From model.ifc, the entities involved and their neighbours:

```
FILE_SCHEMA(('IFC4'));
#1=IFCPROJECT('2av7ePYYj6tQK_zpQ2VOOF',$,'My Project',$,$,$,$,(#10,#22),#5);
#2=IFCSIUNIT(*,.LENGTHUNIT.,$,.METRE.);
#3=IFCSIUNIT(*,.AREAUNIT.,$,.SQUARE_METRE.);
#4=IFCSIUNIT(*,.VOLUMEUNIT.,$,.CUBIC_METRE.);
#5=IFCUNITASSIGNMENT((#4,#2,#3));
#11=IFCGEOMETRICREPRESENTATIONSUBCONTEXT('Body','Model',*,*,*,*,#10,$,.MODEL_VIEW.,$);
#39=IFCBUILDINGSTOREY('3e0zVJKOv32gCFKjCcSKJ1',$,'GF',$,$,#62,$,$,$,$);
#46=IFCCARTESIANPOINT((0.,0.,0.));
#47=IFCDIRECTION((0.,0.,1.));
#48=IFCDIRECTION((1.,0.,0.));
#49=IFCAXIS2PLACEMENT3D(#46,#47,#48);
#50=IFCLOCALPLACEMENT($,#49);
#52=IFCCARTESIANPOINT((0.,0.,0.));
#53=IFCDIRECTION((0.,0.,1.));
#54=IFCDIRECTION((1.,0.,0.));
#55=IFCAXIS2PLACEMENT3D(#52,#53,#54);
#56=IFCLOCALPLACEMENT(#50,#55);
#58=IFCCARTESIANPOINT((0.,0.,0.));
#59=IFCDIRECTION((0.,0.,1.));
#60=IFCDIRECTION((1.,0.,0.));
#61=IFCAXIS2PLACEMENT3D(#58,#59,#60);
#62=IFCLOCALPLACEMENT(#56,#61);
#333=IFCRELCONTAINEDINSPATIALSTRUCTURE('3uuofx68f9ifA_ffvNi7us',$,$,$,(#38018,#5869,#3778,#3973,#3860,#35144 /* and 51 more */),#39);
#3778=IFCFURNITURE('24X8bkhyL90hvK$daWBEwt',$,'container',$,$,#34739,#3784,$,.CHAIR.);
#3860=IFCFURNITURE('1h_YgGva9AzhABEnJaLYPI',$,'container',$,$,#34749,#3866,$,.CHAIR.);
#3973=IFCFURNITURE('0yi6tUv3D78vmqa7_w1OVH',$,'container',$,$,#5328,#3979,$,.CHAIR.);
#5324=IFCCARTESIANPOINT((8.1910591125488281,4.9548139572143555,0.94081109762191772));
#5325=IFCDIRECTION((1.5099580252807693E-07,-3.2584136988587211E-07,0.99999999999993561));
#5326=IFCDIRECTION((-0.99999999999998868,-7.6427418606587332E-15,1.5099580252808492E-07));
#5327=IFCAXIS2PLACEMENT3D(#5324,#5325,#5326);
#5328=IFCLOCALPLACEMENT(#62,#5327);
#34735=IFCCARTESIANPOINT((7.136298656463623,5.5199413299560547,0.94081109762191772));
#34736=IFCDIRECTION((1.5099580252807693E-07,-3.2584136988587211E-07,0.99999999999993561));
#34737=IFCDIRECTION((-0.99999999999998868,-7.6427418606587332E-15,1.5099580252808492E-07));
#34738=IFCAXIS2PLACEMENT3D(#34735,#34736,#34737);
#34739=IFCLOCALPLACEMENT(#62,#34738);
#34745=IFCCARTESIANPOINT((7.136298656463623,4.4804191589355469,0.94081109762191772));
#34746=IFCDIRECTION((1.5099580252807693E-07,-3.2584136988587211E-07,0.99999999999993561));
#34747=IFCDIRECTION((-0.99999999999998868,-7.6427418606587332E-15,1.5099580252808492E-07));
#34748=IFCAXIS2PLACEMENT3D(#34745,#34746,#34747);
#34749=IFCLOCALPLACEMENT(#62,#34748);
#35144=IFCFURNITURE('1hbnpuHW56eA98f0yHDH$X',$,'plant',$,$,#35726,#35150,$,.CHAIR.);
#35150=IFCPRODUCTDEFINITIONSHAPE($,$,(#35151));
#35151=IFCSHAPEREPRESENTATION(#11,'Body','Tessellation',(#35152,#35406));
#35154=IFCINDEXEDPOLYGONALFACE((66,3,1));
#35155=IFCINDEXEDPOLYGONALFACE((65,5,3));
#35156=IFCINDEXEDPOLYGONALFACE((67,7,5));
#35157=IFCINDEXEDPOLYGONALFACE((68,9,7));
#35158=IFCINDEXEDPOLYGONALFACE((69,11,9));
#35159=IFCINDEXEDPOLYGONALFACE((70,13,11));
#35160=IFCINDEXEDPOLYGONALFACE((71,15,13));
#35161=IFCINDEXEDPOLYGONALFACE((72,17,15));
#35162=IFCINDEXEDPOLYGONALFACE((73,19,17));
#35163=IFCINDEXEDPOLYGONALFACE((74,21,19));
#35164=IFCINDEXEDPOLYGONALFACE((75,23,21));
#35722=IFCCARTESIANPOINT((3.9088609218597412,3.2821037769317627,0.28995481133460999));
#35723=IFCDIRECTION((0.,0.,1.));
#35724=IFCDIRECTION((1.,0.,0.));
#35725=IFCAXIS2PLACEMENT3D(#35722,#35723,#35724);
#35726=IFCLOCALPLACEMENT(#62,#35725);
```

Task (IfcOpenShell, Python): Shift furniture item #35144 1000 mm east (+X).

```python
import ifcopenshell
import ifcopenshell.api.geometry
import ifcopenshell.util.placement
import ifcopenshell.util.unit

model = ifcopenshell.open("model.ifc")
unit_scale = ifcopenshell.util.unit.calculate_unit_scale(model)

item = model.by_guid("1hbnpuHW56eA98f0yHDH$X")
matrix = ifcopenshell.util.placement.get_local_placement(item.ObjectPlacement)
matrix[0, 3] += 1 / unit_scale
ifcopenshell.api.geometry.edit_object_placement(model, product=item, matrix=matrix, is_si=False)

print(ifcopenshell.util.placement.get_local_placement(item.ObjectPlacement).round(3) + 0.0)

model.write("model-out.ifc")
```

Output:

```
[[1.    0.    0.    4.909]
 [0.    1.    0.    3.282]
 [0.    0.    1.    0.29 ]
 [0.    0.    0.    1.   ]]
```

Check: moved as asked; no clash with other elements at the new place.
